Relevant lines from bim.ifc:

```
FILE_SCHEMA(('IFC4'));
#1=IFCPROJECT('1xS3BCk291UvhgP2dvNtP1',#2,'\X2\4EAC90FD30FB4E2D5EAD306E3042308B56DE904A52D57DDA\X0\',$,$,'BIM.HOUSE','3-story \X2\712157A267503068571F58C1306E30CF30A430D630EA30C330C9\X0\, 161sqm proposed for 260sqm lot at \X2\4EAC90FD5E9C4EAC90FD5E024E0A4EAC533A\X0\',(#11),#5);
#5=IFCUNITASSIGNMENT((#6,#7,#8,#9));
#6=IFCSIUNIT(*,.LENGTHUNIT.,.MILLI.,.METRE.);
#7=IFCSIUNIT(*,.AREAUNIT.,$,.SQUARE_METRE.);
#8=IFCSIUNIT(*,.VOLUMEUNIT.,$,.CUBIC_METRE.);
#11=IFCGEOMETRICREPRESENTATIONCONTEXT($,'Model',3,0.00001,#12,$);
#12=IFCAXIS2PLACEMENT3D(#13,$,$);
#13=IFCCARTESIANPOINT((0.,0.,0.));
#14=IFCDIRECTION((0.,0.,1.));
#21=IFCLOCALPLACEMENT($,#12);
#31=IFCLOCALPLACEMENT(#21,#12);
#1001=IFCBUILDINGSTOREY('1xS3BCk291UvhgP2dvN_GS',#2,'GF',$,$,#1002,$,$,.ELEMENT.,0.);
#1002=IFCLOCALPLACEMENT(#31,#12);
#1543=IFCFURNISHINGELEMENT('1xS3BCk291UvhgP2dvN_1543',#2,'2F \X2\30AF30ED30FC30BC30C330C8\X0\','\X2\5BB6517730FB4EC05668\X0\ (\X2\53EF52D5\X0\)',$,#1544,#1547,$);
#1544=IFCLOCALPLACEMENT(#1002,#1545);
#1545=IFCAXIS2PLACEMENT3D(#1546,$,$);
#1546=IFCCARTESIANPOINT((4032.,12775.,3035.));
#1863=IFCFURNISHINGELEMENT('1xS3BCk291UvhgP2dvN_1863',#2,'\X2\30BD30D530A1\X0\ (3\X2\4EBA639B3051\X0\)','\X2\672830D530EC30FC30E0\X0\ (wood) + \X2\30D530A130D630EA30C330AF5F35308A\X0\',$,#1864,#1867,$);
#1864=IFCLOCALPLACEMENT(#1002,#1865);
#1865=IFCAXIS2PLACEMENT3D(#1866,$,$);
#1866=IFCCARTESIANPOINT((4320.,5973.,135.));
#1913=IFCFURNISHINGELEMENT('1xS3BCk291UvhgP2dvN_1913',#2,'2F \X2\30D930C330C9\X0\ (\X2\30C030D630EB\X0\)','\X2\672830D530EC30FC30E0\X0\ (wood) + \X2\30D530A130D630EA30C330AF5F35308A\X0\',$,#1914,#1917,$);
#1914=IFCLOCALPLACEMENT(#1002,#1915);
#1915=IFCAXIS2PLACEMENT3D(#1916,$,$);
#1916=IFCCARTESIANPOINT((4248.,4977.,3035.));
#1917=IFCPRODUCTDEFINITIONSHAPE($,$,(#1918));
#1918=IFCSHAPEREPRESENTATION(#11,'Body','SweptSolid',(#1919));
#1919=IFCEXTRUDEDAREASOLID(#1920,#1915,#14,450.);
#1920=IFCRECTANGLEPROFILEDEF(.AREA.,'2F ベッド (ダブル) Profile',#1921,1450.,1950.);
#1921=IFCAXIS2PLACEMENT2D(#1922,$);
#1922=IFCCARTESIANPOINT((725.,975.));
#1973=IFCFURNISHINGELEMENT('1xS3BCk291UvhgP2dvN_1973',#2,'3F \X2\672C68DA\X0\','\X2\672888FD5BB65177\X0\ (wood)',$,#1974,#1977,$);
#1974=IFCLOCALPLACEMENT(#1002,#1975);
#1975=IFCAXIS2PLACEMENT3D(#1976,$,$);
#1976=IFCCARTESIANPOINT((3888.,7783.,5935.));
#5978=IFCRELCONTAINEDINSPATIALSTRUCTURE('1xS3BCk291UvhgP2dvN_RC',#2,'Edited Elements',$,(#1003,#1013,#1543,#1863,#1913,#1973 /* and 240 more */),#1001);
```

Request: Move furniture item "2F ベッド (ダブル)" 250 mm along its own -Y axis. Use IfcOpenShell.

```python
import ifcopenshell
import ifcopenshell.api.geometry
import ifcopenshell.util.placement

model = ifcopenshell.open("bim.ifc")

item = model.by_id(1913)
matrix = ifcopenshell.util.placement.get_local_placement(item.ObjectPlacement)
matrix[:3, 3] -= matrix[:3, 1] * 250.0
ifcopenshell.api.geometry.edit_object_placement(model, product=item, matrix=matrix, is_si=False)

print(ifcopenshell.util.placement.get_local_placement(item.ObjectPlacement).round(3) + 0.0)

model.write("bim_edited.ifc")
```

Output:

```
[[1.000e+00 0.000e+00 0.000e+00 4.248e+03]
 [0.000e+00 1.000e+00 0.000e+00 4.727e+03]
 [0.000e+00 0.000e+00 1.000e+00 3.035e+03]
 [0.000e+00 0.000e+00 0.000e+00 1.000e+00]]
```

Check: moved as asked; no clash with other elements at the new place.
